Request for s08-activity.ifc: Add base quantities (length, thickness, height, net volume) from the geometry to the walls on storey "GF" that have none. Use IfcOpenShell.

First a look at what the model holds.

```python
import ifcopenshell
import ifcopenshell.util.element
import ifcopenshell.util.unit

model = ifcopenshell.open("s08-activity.ifc")
print(model.schema)
for unit_type in ("LENGTHUNIT", "AREAUNIT", "VOLUMEUNIT"):
    print(unit_type, ifcopenshell.util.unit.calculate_unit_scale(model, unit_type))
storey = next(s for s in model.by_type("IfcBuildingStorey") if s.Name == "GF")
walls = [e for e in ifcopenshell.util.element.get_decomposition(storey) if e.is_a("IfcWall")]
for e in sorted(walls, key=lambda e: e.id()):
    print(e.id(), e.is_a(), e.Name, list(ifcopenshell.util.element.get_psets(e, qtos_only=True)), sep=" | ")
```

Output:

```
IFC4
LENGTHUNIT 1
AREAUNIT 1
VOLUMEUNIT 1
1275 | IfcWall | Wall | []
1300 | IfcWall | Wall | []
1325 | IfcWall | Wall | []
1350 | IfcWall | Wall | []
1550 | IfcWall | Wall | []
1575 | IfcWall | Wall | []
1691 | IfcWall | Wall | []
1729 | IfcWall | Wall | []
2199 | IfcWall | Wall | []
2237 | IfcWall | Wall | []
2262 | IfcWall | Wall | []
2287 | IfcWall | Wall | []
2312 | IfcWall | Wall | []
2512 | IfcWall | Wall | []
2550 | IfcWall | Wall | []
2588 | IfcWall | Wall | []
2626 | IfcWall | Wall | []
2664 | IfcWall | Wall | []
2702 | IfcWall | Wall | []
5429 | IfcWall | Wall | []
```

```python
import ifcopenshell
import ifcopenshell.api.pset
import ifcopenshell.geom
import ifcopenshell.util.element
import ifcopenshell.util.shape
import ifcopenshell.util.unit

model = ifcopenshell.open("s08-activity.ifc")
unit_scale = ifcopenshell.util.unit.calculate_unit_scale(model)
volume_scale = ifcopenshell.util.unit.calculate_unit_scale(model, "VOLUMEUNIT")
settings = ifcopenshell.geom.settings()

storey = next(s for s in model.by_type("IfcBuildingStorey") if s.Name == "GF")
walls = [e for e in ifcopenshell.util.element.get_decomposition(storey) if e.is_a("IfcWall")]

for e in sorted(walls, key=lambda e: e.id()):
    if ifcopenshell.util.element.get_psets(e, qtos_only=True, should_inherit=False):
        continue
    # Geometry comes back in metres, in the element's own axes.
    shape = ifcopenshell.geom.create_shape(settings, e)
    values = {
        "Length": ifcopenshell.util.shape.get_x(shape.geometry) / unit_scale,
        "Width": ifcopenshell.util.shape.get_y(shape.geometry) / unit_scale,
        "Height": ifcopenshell.util.shape.get_z(shape.geometry) / unit_scale,
        "NetVolume": ifcopenshell.util.shape.get_volume(shape.geometry) / volume_scale,
    }
    qto = ifcopenshell.api.pset.add_qto(model, product=e, name="Qto_WallBaseQuantities")
    ifcopenshell.api.pset.edit_qto(model, qto=qto, properties=values)
    print(e.id(), {k: round(v, 3) for k, v in values.items()})

model.write("s08-activity_updated.ifc")
```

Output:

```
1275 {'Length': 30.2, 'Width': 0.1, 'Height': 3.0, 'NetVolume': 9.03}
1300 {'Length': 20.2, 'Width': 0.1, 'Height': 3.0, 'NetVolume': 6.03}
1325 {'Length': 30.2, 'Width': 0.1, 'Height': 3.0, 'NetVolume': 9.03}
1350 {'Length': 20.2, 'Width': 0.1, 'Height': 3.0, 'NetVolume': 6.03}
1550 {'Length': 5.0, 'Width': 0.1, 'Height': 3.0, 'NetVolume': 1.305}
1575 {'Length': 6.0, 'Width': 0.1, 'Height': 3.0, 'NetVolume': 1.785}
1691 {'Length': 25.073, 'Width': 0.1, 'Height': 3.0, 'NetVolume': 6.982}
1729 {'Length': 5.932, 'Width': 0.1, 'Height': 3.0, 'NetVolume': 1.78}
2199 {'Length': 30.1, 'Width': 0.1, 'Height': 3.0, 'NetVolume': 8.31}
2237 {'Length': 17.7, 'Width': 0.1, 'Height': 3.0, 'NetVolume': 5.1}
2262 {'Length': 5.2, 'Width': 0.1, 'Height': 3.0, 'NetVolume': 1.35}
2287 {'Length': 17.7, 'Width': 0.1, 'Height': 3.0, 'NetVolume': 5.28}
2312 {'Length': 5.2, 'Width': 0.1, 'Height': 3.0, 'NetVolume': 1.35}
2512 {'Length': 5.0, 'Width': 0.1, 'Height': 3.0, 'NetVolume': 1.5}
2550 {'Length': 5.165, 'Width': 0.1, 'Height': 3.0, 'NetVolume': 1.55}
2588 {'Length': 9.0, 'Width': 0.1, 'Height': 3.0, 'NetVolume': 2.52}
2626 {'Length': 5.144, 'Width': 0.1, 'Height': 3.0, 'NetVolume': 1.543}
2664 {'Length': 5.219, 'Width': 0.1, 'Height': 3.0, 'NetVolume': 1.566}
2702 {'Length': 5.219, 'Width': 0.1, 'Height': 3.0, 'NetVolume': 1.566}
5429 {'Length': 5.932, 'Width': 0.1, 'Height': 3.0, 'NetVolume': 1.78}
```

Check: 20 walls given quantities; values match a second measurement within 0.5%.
